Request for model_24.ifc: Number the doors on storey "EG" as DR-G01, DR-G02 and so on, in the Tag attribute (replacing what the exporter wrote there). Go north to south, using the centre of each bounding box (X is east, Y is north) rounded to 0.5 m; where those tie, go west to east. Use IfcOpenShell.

First a look at what the model holds.

```python
import ifcopenshell
import ifcopenshell.util.element
import ifcopenshell.util.placement

model = ifcopenshell.open("model_24.ifc")
print(model.schema)
storey = next(s for s in model.by_type("IfcBuildingStorey") if s.Name == "EG")
doors = [e for e in ifcopenshell.util.element.get_decomposition(storey) if e.is_a("IfcDoor")]
for e in sorted(doors, key=lambda e: e.id()):
    origin = ifcopenshell.util.placement.get_local_placement(e.ObjectPlacement)[:3, 3]
    print(e.id(), e.Tag, e.Name, origin.round(2) + 0.0, sep=" | ")
```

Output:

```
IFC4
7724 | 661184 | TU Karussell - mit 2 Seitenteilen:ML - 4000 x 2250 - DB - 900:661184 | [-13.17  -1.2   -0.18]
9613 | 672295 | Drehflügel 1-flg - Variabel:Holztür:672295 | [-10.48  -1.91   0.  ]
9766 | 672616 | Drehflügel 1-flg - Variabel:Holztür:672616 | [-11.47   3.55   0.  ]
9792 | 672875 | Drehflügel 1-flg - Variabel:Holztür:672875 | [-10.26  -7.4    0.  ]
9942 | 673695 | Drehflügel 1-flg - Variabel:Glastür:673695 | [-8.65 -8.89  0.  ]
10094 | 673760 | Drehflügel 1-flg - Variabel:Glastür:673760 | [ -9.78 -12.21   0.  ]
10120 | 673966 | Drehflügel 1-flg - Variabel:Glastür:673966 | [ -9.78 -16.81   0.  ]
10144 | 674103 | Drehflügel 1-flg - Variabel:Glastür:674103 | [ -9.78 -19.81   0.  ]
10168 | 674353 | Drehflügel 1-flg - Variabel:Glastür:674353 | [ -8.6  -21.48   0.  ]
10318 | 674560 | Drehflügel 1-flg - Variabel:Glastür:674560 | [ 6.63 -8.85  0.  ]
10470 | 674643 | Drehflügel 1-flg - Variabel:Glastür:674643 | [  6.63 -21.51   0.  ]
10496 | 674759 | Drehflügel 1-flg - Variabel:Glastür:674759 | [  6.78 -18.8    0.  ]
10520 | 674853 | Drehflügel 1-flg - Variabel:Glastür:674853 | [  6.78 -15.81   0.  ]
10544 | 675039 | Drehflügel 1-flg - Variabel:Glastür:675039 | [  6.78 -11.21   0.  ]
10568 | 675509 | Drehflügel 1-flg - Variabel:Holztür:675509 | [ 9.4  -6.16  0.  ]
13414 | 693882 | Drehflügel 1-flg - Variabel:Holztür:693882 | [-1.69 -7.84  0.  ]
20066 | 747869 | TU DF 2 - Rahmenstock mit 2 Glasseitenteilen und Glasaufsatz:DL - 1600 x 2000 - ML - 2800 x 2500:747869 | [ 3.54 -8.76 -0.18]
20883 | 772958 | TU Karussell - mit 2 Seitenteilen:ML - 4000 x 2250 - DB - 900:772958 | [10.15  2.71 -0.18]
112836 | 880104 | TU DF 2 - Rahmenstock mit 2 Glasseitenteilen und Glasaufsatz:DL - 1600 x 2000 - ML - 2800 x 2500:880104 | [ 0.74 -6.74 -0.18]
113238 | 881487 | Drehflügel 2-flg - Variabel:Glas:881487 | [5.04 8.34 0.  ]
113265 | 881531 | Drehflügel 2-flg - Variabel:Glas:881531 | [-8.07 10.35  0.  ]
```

```python
import ifcopenshell
import ifcopenshell.geom
import ifcopenshell.util.element
import ifcopenshell.util.shape

model = ifcopenshell.open("model_24.ifc")
settings = ifcopenshell.geom.settings()
settings.set("use-world-coords", True)


def centre(element):
    shape = ifcopenshell.geom.create_shape(settings, element)
    return ifcopenshell.util.shape.get_bbox_centroid(shape.geometry)


storey = next(s for s in model.by_type("IfcBuildingStorey") if s.Name == "EG")
doors = [e for e in ifcopenshell.util.element.get_decomposition(storey) if e.is_a("IfcDoor")]

# Insertion points can sit at a corner or the storey origin, so sort by the geometry (in metres).
centres = {e: centre(e) for e in doors}
doors.sort(key=lambda e: (-round(centres[e][1] / 0.5), centres[e][0]))

for i, e in enumerate(doors, start=1):
    number = f"DR-G{i:02d}"
    e.Tag = number
    print(e.id(), number)

model.write("model_24_rev.ifc")
```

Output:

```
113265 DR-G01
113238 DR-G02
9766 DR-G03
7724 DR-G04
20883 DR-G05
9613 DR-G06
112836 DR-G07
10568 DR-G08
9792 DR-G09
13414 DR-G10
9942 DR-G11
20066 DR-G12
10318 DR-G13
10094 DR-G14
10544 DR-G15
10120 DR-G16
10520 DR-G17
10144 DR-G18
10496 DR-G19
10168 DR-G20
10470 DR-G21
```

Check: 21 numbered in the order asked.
